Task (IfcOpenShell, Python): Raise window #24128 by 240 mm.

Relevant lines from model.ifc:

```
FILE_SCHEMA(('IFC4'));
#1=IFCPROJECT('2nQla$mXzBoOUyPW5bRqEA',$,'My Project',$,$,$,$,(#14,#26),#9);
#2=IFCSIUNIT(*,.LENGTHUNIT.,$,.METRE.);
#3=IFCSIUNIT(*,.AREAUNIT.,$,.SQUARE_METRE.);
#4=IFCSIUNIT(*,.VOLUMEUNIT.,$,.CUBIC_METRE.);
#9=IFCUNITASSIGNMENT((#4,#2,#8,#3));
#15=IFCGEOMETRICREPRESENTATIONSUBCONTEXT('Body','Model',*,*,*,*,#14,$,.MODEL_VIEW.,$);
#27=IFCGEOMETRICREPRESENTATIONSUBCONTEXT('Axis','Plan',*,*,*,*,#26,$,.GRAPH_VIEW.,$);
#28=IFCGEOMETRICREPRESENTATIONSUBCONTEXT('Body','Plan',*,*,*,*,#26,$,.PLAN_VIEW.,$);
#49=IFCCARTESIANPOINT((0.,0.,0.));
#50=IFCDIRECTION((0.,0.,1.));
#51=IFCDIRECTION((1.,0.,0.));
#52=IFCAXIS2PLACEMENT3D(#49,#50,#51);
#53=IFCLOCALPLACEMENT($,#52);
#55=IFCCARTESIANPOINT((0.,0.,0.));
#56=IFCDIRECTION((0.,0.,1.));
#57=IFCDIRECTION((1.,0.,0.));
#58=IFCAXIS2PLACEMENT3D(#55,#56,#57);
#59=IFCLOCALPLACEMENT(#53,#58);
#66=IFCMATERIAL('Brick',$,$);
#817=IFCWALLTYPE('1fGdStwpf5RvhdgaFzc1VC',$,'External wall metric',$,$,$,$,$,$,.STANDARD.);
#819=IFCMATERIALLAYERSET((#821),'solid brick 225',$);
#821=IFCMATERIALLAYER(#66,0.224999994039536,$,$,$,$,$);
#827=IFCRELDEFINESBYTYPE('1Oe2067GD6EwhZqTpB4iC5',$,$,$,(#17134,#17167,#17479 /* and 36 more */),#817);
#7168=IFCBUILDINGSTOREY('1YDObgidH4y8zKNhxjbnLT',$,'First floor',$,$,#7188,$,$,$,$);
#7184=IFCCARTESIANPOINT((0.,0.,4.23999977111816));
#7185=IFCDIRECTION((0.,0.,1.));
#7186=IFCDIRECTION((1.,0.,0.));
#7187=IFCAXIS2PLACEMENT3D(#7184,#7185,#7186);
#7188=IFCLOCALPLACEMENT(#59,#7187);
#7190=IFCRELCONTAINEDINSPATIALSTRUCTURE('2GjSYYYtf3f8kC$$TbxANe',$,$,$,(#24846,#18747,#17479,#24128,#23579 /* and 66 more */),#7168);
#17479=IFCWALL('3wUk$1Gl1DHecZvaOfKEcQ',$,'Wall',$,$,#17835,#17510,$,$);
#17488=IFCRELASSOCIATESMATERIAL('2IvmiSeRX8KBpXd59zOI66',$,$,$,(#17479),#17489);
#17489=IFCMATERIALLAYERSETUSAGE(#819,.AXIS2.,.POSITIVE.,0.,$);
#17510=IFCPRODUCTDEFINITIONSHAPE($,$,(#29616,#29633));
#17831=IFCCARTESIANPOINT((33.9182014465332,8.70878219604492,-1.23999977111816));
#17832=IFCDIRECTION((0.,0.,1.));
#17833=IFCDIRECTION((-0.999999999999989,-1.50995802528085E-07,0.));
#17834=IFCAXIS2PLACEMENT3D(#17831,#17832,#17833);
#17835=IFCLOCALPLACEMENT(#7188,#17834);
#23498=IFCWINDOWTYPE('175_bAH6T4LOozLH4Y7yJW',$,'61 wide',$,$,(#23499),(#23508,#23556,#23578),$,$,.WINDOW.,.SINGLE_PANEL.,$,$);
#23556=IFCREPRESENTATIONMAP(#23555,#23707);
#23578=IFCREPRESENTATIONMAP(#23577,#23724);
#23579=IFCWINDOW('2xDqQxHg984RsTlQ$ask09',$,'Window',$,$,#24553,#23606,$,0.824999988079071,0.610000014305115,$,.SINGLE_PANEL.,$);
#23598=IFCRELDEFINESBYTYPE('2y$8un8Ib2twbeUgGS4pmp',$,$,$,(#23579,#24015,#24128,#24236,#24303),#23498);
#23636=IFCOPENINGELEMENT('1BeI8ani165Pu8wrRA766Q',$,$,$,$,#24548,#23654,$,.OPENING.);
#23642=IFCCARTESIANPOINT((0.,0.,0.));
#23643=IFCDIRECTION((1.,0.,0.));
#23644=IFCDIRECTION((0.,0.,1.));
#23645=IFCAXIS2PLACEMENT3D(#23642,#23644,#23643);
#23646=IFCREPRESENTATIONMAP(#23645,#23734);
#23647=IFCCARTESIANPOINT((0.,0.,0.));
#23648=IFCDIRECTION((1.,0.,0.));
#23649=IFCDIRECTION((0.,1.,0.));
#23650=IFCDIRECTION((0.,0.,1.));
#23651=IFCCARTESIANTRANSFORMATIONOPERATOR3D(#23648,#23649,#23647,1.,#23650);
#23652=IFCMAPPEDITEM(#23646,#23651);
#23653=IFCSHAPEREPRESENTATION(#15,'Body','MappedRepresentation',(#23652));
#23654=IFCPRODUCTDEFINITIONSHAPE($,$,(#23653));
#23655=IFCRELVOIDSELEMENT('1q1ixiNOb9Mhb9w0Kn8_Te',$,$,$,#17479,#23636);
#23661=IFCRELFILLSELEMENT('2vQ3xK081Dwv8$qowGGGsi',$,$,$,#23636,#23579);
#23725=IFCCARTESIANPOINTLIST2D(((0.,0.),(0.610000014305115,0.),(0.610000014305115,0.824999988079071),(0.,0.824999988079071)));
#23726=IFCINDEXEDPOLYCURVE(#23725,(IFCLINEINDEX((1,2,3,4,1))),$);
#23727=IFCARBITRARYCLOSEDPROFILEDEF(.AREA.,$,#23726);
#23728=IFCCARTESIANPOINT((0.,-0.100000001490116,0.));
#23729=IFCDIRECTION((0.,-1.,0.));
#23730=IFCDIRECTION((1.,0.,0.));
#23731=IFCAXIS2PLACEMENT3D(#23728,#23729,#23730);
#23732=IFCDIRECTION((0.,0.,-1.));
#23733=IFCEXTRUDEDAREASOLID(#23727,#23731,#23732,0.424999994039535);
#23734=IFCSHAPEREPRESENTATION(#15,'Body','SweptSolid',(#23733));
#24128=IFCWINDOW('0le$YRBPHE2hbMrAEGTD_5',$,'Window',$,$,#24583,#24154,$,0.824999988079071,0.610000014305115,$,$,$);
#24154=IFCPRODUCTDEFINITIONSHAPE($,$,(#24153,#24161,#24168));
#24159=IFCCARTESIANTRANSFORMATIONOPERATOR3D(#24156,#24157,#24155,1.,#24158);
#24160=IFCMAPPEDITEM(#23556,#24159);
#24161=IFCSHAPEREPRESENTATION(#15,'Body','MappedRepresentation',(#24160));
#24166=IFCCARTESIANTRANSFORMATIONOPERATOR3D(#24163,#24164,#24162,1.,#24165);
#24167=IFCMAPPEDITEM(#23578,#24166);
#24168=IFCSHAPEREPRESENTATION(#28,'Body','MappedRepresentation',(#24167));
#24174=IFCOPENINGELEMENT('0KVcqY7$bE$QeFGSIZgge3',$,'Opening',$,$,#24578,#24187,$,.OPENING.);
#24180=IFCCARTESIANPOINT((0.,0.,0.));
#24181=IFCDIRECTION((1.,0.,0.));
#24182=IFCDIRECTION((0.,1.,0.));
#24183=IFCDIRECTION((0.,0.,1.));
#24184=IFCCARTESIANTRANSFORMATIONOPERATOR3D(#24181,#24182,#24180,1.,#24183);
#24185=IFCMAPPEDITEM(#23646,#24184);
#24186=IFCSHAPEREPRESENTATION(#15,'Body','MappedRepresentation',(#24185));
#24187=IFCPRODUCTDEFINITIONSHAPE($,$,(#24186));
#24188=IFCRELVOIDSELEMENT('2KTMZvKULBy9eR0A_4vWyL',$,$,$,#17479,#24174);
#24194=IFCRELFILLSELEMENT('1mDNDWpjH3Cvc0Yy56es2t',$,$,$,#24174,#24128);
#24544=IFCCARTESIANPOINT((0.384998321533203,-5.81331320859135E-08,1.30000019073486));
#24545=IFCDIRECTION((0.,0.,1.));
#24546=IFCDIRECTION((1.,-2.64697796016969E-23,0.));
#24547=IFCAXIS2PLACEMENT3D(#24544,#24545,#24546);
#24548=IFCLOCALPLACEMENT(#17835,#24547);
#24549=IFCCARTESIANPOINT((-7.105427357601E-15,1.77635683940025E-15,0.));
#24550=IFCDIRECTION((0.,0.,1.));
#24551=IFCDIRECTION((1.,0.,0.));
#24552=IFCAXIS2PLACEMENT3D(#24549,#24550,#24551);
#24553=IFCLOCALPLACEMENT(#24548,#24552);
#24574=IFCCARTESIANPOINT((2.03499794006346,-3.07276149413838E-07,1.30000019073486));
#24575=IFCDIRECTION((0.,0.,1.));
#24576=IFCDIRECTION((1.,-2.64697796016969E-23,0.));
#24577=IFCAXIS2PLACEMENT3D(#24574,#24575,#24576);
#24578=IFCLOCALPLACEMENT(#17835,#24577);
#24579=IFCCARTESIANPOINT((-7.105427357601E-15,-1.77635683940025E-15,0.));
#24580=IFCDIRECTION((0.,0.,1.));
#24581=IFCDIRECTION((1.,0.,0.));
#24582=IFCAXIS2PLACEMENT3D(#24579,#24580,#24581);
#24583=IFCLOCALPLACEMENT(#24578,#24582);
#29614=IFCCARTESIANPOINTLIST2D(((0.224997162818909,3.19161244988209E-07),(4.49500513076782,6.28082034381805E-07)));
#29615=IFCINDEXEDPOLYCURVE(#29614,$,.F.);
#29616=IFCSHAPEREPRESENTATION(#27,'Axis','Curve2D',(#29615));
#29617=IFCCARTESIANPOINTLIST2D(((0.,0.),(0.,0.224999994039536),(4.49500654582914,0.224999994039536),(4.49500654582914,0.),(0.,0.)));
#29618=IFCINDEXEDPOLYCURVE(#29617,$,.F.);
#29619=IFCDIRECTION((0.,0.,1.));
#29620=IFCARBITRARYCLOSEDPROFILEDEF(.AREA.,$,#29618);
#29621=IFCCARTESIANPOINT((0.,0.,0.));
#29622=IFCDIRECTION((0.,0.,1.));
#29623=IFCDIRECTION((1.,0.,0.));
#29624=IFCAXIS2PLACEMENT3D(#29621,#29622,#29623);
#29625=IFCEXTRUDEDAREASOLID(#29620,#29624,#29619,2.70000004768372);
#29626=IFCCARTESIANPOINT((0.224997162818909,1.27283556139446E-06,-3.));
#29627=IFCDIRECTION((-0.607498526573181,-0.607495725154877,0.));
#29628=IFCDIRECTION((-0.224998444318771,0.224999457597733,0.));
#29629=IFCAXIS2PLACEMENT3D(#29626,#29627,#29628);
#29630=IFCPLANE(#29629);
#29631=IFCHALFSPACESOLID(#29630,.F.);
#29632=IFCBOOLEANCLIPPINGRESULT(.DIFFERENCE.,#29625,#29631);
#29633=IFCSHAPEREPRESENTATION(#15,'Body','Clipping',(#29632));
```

```python
import numpy as np
import ifcopenshell
import ifcopenshell.api.geometry
import ifcopenshell.util.placement
import ifcopenshell.util.unit

model = ifcopenshell.open("model.ifc")
unit_scale = ifcopenshell.util.unit.calculate_unit_scale(model)

window = model.by_guid("0le$YRBPHE2hbMrAEGTD_5")
opening = window.FillsVoids[0].RelatingOpeningElement
dz = 0.24 / unit_scale

shift = np.array([0.0, 0.0, dz])
# The window is placed relative to its opening, so it follows when the opening moves.
matrix = ifcopenshell.util.placement.get_local_placement(opening.ObjectPlacement)
matrix[:3, 3] += shift
ifcopenshell.api.geometry.edit_object_placement(
    model, product=opening, matrix=matrix, is_si=False, should_transform_children=True
)

print(f"moved by {dz * unit_scale:+.3f} m")

model.write("model_rev.ifc")
```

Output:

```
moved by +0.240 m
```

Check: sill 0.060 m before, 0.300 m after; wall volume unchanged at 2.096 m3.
